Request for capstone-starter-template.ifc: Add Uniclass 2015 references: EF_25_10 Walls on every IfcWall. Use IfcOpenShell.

First a look at what the model holds.

```python
import ifcopenshell

model = ifcopenshell.open("capstone-starter-template.ifc")
print(model.schema)
print("classifications:", [c.Name for c in model.by_type("IfcClassification")])
for ifc_class in ("IfcDoor", "IfcRoof", "IfcStair", "IfcWall", "IfcWindow"):
    print(ifc_class, len(model.by_type(ifc_class)))
```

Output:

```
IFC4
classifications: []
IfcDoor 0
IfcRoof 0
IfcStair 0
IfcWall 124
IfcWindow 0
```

```python
import ifcopenshell
import ifcopenshell.api.classification

model = ifcopenshell.open("capstone-starter-template.ifc")

system = ifcopenshell.api.classification.add_classification(model, classification="Uniclass 2015")

codes = {
    "IfcWall": ("EF_25_10", "Walls"),
}
for ifc_class, (code, name) in codes.items():
    products = model.by_type(ifc_class)
    ifcopenshell.api.classification.add_reference(
        model, products=products, classification=system, identification=code, name=name
    )
    print(code, len(products))

model.write("capstone-starter-template-out.ifc")
```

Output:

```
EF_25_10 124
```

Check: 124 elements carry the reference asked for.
